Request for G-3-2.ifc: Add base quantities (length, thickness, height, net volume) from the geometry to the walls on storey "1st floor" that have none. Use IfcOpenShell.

First a look at what the model holds.

```python
import ifcopenshell
import ifcopenshell.util.element
import ifcopenshell.util.unit

model = ifcopenshell.open("G-3-2.ifc")
print(model.schema)
for unit_type in ("LENGTHUNIT", "AREAUNIT", "VOLUMEUNIT"):
    print(unit_type, ifcopenshell.util.unit.calculate_unit_scale(model, unit_type))
storey = next(s for s in model.by_type("IfcBuildingStorey") if s.Name == "1st floor")
walls = [e for e in ifcopenshell.util.element.get_decomposition(storey) if e.is_a("IfcWall")]
for e in sorted(walls, key=lambda e: e.id()):
    print(e.id(), e.is_a(), e.Name, list(ifcopenshell.util.element.get_psets(e, qtos_only=True)), sep=" | ")
```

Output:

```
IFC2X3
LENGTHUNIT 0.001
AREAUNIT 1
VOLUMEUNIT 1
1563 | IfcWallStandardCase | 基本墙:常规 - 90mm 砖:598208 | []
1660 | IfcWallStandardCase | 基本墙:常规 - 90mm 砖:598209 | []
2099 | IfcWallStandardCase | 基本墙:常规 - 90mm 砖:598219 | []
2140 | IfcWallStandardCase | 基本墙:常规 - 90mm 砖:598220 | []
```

```python
import ifcopenshell
import ifcopenshell.api.pset
import ifcopenshell.geom
import ifcopenshell.util.element
import ifcopenshell.util.shape
import ifcopenshell.util.unit

model = ifcopenshell.open("G-3-2.ifc")
unit_scale = ifcopenshell.util.unit.calculate_unit_scale(model)
volume_scale = ifcopenshell.util.unit.calculate_unit_scale(model, "VOLUMEUNIT")
settings = ifcopenshell.geom.settings()

storey = next(s for s in model.by_type("IfcBuildingStorey") if s.Name == "1st floor")
walls = [e for e in ifcopenshell.util.element.get_decomposition(storey) if e.is_a("IfcWall")]

for e in sorted(walls, key=lambda e: e.id()):
    if ifcopenshell.util.element.get_psets(e, qtos_only=True, should_inherit=False):
        continue
    # Geometry comes back in metres, in the element's own axes.
    shape = ifcopenshell.geom.create_shape(settings, e)
    values = {
        "Length": ifcopenshell.util.shape.get_x(shape.geometry) / unit_scale,
        "Width": ifcopenshell.util.shape.get_y(shape.geometry) / unit_scale,
        "Height": ifcopenshell.util.shape.get_z(shape.geometry) / unit_scale,
        "NetVolume": ifcopenshell.util.shape.get_volume(shape.geometry) / volume_scale,
    }
    qto = ifcopenshell.api.pset.add_qto(model, product=e, name="BaseQuantities")
    ifcopenshell.api.pset.edit_qto(model, qto=qto, properties=values)
    print(e.id(), {k: round(v, 3) for k, v in values.items()})

model.write("G-3-2_updated.ifc")
```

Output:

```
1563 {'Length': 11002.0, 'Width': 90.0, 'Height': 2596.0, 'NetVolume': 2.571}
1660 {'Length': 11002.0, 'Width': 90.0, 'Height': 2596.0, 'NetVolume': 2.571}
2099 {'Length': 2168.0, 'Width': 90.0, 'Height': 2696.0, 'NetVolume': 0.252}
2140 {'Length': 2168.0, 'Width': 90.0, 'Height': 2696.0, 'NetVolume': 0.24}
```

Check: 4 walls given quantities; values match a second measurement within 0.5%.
